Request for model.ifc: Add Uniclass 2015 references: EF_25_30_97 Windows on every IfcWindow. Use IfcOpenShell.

First a look at what the model holds.

```python
import ifcopenshell

model = ifcopenshell.open("model.ifc")
print(model.schema)
print("classifications:", [c.Name for c in model.by_type("IfcClassification")])
for ifc_class in ("IfcDoor", "IfcRoof", "IfcStair", "IfcWall", "IfcWindow"):
    print(ifc_class, len(model.by_type(ifc_class)))
```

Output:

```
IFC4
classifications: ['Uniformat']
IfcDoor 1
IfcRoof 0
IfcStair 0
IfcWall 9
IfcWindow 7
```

```python
import ifcopenshell
import ifcopenshell.api.classification

model = ifcopenshell.open("model.ifc")

system = ifcopenshell.api.classification.add_classification(model, classification="Uniclass 2015")

codes = {
    "IfcWindow": ("EF_25_30_97", "Windows"),
}
for ifc_class, (code, name) in codes.items():
    products = model.by_type(ifc_class)
    ifcopenshell.api.classification.add_reference(
        model, products=products, classification=system, identification=code, name=name
    )
    print(code, len(products))

model.write("model_rev.ifc")
```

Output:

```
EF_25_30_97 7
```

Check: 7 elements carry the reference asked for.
